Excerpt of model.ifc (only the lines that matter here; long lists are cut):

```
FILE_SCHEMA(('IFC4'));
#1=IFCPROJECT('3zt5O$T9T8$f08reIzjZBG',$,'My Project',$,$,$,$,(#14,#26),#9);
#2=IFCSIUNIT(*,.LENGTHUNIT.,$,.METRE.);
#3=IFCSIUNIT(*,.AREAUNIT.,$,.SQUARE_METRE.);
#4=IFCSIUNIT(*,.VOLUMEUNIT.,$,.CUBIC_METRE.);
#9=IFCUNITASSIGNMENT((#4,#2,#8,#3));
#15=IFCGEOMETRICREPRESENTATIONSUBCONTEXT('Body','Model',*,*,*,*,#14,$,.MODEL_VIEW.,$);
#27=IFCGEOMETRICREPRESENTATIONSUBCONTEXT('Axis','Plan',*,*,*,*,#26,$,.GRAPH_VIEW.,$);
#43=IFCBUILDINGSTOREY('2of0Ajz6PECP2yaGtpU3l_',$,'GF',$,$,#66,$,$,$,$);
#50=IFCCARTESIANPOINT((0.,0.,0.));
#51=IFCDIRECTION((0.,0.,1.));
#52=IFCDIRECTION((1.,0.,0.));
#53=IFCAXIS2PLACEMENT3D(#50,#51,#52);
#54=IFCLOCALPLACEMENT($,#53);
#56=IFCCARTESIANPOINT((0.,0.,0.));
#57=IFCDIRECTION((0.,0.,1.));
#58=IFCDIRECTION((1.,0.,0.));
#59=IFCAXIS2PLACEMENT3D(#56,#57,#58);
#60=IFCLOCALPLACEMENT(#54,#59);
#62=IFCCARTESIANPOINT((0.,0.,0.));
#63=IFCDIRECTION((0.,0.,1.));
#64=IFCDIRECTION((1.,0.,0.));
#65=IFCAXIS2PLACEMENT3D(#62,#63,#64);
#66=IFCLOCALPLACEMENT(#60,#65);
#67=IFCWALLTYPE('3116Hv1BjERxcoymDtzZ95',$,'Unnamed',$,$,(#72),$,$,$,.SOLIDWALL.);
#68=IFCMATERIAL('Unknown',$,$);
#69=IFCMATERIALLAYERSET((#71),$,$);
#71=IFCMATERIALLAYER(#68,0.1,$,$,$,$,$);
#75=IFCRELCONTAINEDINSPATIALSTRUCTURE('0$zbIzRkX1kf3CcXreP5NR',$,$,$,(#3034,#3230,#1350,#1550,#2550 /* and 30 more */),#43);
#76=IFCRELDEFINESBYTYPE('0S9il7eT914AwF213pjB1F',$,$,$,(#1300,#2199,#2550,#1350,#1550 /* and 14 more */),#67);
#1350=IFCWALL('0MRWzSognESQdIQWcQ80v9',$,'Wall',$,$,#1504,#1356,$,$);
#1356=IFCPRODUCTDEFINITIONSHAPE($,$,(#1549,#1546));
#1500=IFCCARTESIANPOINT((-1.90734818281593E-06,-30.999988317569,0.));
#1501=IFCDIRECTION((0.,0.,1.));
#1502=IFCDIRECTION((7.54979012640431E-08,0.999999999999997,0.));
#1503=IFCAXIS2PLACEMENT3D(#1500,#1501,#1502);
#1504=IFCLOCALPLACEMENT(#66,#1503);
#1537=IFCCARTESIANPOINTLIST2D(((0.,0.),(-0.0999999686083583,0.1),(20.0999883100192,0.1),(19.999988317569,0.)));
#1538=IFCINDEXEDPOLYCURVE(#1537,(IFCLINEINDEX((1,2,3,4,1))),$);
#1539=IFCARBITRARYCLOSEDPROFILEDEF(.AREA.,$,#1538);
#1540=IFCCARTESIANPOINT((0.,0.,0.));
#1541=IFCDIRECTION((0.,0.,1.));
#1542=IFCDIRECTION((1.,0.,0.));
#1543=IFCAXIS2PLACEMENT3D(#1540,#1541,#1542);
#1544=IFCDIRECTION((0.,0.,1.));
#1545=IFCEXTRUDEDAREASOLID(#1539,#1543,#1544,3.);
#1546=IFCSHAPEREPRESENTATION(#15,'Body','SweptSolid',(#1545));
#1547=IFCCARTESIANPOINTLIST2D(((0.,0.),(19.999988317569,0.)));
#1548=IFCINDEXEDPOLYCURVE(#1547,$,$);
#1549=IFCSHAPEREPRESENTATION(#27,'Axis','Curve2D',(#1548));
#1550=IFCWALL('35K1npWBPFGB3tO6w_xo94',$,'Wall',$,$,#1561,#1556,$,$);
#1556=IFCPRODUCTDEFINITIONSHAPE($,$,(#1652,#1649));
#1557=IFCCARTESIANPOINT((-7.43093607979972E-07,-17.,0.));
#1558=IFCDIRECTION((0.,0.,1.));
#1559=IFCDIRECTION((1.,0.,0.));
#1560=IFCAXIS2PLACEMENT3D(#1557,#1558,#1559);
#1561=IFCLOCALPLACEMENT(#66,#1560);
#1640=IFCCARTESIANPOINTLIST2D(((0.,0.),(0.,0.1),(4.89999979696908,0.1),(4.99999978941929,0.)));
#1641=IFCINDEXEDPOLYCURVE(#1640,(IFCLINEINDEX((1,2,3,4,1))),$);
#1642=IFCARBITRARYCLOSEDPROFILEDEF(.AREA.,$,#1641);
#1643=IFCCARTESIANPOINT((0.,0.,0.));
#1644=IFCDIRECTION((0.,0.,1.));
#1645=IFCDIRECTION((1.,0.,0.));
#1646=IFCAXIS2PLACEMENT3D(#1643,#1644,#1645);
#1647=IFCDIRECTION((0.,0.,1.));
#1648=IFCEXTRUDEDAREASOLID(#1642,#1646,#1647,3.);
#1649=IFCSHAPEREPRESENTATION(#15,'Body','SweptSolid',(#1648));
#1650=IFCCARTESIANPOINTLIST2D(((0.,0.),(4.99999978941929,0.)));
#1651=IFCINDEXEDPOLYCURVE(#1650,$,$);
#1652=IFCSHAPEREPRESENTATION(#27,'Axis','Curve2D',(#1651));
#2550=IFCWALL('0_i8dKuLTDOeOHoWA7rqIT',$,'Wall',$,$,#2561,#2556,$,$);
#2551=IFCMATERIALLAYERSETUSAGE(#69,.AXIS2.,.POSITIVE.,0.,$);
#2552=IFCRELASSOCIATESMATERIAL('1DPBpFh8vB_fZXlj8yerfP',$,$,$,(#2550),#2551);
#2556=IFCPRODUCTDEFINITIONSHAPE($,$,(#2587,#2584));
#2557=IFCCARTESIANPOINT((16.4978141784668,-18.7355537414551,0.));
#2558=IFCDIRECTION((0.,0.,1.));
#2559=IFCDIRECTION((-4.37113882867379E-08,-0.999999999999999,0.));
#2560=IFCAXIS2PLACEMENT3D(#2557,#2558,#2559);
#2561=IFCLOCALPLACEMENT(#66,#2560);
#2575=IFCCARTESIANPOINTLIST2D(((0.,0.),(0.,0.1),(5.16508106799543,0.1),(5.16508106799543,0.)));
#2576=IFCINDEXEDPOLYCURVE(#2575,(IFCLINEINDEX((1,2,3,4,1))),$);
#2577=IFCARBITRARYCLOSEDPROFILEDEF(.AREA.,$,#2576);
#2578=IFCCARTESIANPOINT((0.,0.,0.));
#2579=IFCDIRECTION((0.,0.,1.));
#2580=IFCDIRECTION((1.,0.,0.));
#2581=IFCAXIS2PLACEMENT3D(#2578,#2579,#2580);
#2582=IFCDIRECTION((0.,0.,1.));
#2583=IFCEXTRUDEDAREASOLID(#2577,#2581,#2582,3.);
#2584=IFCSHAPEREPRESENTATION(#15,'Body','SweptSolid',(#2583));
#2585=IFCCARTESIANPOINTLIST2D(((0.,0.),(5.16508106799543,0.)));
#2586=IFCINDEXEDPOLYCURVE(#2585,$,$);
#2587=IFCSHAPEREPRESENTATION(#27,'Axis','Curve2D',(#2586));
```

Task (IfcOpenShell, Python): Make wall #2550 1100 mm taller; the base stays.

```python
import ifcopenshell
import ifcopenshell.geom
import ifcopenshell.util.representation
import ifcopenshell.util.shape

model = ifcopenshell.open("model.ifc")
settings = ifcopenshell.geom.settings()


def volume(element):
    """Net volume in cubic metres, openings subtracted."""
    shape = ifcopenshell.geom.create_shape(settings, element)
    return ifcopenshell.util.shape.get_volume(shape.geometry)


wall = model.by_guid("0_i8dKuLTDOeOHoWA7rqIT")
before = volume(wall)

body = ifcopenshell.util.representation.get_representation(wall, "Model", "Body")
solid = body.Items[0]
old_height = solid.Depth
solid.Depth += 1.1
after = volume(wall)

print(f"height {old_height:g} -> {solid.Depth:g}, volume {before:.3f} -> {after:.3f} m3")

model.write("model_updated.ifc")
```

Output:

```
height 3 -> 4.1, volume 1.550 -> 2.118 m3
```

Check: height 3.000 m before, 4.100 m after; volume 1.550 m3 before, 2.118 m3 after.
